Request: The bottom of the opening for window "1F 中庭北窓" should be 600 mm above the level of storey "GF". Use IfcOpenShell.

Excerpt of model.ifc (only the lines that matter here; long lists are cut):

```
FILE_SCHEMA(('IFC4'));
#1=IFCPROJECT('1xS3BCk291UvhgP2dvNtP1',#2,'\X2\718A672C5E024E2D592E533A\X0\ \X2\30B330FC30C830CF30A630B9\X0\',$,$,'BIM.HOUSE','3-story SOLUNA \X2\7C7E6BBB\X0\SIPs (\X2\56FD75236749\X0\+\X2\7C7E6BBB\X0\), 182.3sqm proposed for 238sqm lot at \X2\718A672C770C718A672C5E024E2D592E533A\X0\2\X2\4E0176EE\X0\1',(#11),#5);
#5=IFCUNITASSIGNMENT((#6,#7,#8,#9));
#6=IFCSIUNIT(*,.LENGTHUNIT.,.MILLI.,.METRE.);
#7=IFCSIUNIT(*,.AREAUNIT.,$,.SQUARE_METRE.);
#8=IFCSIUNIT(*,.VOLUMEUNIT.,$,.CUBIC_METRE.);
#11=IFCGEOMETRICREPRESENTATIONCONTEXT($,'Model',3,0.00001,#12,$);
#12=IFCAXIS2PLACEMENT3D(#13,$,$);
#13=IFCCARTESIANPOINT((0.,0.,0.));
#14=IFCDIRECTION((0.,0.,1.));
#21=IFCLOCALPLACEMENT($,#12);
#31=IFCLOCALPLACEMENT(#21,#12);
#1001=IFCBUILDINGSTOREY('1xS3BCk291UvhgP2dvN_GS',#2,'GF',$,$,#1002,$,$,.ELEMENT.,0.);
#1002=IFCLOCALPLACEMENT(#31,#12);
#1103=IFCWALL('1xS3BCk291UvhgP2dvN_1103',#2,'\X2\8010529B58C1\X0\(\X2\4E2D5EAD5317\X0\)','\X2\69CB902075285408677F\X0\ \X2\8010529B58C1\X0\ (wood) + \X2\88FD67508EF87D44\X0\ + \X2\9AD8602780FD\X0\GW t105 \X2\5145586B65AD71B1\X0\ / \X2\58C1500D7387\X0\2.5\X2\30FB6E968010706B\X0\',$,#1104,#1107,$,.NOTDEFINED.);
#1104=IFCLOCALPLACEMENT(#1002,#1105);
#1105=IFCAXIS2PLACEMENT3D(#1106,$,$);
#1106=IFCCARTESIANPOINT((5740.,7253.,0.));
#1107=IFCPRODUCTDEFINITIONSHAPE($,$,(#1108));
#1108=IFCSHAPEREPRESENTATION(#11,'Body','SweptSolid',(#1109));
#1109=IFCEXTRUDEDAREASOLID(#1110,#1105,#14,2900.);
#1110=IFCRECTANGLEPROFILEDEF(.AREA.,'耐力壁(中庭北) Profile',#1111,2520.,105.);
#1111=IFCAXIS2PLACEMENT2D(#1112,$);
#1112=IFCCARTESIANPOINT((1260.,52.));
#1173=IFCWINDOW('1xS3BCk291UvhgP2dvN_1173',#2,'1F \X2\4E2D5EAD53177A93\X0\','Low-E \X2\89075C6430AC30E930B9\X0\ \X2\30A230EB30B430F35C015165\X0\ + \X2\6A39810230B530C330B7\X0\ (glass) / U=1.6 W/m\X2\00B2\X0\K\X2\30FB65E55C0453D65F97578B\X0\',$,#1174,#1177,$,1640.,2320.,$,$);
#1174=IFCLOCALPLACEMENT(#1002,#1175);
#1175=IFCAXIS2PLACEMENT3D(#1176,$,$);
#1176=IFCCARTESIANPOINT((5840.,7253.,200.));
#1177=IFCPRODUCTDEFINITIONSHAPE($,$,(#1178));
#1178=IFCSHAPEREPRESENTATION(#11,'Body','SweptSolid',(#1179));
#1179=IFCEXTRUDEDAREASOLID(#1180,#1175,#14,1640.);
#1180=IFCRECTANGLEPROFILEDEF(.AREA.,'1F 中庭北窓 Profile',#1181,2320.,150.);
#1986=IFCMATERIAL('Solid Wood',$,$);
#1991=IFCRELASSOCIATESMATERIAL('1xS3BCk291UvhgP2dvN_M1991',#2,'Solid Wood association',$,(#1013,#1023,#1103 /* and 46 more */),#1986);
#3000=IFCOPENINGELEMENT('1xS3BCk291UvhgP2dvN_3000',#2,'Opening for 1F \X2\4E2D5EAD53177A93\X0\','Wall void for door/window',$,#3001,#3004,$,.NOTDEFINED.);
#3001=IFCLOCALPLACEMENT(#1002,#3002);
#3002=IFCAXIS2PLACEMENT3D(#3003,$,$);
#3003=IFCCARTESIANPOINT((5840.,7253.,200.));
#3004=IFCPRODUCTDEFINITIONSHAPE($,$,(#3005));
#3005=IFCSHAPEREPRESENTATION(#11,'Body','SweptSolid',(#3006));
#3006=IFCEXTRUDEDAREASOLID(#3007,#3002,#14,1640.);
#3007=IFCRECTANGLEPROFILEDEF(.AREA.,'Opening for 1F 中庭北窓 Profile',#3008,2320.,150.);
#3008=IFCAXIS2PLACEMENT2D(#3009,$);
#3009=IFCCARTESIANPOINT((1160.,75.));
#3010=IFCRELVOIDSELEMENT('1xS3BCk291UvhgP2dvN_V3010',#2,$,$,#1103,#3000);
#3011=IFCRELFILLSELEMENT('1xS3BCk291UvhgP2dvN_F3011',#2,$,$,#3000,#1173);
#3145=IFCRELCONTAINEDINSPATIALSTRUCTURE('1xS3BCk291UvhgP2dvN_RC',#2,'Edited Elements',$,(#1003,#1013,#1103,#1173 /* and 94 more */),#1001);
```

```python
import numpy as np
import ifcopenshell
import ifcopenshell.api.geometry
import ifcopenshell.geom
import ifcopenshell.util.element
import ifcopenshell.util.placement
import ifcopenshell.util.shape
import ifcopenshell.util.unit

model = ifcopenshell.open("model.ifc")
unit_scale = ifcopenshell.util.unit.calculate_unit_scale(model)

window = model.by_guid("1xS3BCk291UvhgP2dvN_1173")
opening = window.FillsVoids[0].RelatingOpeningElement
storey = ifcopenshell.util.element.get_container(window, ifc_class="IfcBuildingStorey")
level = ifcopenshell.util.placement.get_local_placement(storey.ObjectPlacement)[2, 3]

# The opening's origin need not be at the sill, so measure its lowest point.
shape = ifcopenshell.geom.create_shape(ifcopenshell.geom.settings(), opening)
bottom = ifcopenshell.util.shape.get_shape_bottom_elevation(shape, shape.geometry) / unit_scale
dz = level + 600.0 - bottom

shift = np.array([0.0, 0.0, dz])
# The window is not placed relative to its opening, so move both.
for product in (opening, window):
    matrix = ifcopenshell.util.placement.get_local_placement(product.ObjectPlacement)
    matrix[:3, 3] += shift
    ifcopenshell.api.geometry.edit_object_placement(model, product=product, matrix=matrix, is_si=False)

print(f"moved by {dz * unit_scale:+.3f} m")

model.write("model_v2.ifc")
```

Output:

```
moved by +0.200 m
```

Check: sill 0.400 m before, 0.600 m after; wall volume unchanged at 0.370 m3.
